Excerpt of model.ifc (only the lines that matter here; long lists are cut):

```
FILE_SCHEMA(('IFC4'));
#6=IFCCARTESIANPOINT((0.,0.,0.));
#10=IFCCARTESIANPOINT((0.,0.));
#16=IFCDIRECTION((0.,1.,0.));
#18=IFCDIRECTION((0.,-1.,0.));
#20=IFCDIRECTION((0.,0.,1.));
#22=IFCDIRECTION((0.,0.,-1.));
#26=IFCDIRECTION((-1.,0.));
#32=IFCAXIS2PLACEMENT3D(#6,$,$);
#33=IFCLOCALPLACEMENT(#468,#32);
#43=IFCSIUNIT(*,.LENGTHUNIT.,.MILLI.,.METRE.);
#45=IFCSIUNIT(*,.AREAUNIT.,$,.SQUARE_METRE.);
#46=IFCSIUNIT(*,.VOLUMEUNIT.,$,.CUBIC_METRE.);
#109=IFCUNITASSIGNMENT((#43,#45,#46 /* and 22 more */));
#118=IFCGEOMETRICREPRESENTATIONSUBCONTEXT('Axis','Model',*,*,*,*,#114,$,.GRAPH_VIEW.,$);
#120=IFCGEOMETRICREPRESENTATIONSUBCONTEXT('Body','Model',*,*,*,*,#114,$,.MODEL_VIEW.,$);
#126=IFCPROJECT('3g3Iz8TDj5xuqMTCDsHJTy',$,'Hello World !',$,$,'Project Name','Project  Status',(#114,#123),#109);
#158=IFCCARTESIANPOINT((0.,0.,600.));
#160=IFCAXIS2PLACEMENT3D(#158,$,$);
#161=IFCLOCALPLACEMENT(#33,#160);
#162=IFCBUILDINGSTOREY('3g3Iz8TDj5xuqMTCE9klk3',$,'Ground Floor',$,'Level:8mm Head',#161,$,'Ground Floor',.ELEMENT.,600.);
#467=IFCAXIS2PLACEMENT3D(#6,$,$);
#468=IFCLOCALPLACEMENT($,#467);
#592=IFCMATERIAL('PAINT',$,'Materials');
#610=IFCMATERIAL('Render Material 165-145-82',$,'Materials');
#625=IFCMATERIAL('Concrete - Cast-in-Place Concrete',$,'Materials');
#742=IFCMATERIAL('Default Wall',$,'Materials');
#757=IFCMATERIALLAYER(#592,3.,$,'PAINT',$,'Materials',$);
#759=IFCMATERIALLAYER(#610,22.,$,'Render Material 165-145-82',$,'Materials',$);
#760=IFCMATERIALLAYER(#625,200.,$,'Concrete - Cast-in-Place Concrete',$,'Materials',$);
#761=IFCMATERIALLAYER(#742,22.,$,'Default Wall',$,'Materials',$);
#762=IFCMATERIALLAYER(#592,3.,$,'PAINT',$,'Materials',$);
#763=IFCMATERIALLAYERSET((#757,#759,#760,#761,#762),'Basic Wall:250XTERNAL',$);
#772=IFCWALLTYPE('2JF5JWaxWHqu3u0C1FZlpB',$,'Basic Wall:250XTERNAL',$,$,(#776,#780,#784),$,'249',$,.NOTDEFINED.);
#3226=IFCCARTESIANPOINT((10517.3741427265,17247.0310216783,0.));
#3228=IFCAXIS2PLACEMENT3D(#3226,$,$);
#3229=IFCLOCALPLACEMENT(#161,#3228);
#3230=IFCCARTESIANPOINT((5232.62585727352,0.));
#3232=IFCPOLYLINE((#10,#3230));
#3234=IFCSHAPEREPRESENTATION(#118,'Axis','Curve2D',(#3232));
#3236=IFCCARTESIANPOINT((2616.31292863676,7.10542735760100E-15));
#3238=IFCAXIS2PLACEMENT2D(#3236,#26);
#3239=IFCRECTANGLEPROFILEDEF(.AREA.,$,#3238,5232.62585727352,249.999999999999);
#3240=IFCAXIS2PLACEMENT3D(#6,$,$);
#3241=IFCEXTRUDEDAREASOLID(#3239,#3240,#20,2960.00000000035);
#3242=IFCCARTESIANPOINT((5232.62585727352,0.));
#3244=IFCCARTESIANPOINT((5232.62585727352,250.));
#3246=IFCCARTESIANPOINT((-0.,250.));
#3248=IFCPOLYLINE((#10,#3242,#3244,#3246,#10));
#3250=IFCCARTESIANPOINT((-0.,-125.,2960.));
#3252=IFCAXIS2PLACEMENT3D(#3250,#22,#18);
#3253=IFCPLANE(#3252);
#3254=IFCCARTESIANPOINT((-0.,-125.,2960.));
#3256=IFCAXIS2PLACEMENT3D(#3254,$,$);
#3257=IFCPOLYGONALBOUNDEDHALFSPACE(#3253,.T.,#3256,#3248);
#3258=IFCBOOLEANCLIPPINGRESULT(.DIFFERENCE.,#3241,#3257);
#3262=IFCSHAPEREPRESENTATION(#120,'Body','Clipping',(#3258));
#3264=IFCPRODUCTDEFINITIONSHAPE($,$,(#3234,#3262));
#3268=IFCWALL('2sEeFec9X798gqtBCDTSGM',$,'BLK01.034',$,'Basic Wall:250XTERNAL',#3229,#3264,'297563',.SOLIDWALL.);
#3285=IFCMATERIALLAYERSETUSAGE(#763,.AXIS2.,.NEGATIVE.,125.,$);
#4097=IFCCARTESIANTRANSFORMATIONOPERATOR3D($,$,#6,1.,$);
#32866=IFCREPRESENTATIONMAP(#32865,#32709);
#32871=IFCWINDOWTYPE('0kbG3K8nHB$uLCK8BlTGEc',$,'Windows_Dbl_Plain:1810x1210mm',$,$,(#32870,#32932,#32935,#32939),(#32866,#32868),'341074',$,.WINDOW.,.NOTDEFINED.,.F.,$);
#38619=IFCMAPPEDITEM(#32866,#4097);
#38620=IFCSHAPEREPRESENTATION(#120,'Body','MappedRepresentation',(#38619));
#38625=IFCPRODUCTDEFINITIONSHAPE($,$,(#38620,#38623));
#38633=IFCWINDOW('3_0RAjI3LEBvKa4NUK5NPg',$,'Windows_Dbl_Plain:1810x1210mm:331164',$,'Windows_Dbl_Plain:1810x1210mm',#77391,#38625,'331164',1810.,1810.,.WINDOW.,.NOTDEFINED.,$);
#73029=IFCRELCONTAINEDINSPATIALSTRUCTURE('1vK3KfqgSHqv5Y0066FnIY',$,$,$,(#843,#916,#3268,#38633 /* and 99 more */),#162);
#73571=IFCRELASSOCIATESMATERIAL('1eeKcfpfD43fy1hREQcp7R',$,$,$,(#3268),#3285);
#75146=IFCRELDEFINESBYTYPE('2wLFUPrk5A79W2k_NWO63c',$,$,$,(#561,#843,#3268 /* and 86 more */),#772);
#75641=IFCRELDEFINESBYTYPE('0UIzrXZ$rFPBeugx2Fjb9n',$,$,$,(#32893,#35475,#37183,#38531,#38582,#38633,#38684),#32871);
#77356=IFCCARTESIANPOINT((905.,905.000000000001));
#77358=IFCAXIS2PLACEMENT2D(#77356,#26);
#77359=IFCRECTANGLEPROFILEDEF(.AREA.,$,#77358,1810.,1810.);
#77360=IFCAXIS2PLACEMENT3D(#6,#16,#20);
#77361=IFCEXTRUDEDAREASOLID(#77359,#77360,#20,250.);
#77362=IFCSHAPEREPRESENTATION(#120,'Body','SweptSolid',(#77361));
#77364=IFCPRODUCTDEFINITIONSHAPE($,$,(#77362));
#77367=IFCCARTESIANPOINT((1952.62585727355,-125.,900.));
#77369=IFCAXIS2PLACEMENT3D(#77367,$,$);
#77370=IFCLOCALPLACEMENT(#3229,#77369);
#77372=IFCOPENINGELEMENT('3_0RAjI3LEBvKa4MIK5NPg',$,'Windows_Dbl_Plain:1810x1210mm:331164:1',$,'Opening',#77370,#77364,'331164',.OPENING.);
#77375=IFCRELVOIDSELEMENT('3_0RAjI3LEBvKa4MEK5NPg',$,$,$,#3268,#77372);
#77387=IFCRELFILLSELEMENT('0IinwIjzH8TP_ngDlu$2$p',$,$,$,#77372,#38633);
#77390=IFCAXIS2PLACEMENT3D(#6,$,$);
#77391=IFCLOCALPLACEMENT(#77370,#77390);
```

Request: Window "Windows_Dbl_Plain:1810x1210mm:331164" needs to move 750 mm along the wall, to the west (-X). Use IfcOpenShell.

```python
import ifcopenshell
import ifcopenshell.api.geometry
import ifcopenshell.util.placement

model = ifcopenshell.open("model.ifc")

window = model.by_guid("3_0RAjI3LEBvKa4NUK5NPg")
opening = window.FillsVoids[0].RelatingOpeningElement
wall = opening.VoidsElements[0].RelatingBuildingElement

wall_matrix = ifcopenshell.util.placement.get_local_placement(wall.ObjectPlacement)
shift = wall_matrix[:3, 0] * -750.0
before = ifcopenshell.util.placement.get_local_placement(window.ObjectPlacement)[:3, 3].copy()

# The window is placed relative to its opening, so it follows when the opening moves.
matrix = ifcopenshell.util.placement.get_local_placement(opening.ObjectPlacement)
matrix[:3, 3] += shift
ifcopenshell.api.geometry.edit_object_placement(
    model, product=opening, matrix=matrix, is_si=False, should_transform_children=True
)

after = ifcopenshell.util.placement.get_local_placement(window.ObjectPlacement)[:3, 3]
print("window moved by", (after - before).round(3) + 0.0)

model.write("model-out.ifc")
```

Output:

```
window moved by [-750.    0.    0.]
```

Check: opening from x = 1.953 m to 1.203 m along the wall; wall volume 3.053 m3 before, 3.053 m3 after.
